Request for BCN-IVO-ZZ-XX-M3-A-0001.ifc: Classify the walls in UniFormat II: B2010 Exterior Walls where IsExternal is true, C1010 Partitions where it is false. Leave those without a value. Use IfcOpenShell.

First a look at what the model holds.

```python
import ifcopenshell
import ifcopenshell.util.element

model = ifcopenshell.open("BCN-IVO-ZZ-XX-M3-A-0001.ifc")
print(model.schema)
print("classifications:", [c.Name for c in model.by_type("IfcClassification")])
values = [ifcopenshell.util.element.get_pset(e, "Pset_WallCommon", "IsExternal") for e in model.by_type("IfcWall")]
for value in (True, False, None):
    print("IsExternal", value, values.count(value))
```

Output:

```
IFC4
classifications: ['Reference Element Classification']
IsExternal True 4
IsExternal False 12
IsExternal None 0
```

```python
import ifcopenshell
import ifcopenshell.api.classification
import ifcopenshell.util.element

model = ifcopenshell.open("BCN-IVO-ZZ-XX-M3-A-0001.ifc")

system = ifcopenshell.api.classification.add_classification(model, classification="UniFormat II")

walls = model.by_type("IfcWall")
external = {e: ifcopenshell.util.element.get_pset(e, "Pset_WallCommon", "IsExternal") for e in walls}
for flag, code, name in ((True, "B2010", "Exterior Walls"), (False, "C1010", "Partitions")):
    products = [e for e in walls if external[e] is flag]
    ifcopenshell.api.classification.add_reference(
        model, products=products, classification=system, identification=code, name=name
    )
    print(code, len(products))

model.write("BCN-IVO-ZZ-XX-M3-A-0001_edited.ifc")
```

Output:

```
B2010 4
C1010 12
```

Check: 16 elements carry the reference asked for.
